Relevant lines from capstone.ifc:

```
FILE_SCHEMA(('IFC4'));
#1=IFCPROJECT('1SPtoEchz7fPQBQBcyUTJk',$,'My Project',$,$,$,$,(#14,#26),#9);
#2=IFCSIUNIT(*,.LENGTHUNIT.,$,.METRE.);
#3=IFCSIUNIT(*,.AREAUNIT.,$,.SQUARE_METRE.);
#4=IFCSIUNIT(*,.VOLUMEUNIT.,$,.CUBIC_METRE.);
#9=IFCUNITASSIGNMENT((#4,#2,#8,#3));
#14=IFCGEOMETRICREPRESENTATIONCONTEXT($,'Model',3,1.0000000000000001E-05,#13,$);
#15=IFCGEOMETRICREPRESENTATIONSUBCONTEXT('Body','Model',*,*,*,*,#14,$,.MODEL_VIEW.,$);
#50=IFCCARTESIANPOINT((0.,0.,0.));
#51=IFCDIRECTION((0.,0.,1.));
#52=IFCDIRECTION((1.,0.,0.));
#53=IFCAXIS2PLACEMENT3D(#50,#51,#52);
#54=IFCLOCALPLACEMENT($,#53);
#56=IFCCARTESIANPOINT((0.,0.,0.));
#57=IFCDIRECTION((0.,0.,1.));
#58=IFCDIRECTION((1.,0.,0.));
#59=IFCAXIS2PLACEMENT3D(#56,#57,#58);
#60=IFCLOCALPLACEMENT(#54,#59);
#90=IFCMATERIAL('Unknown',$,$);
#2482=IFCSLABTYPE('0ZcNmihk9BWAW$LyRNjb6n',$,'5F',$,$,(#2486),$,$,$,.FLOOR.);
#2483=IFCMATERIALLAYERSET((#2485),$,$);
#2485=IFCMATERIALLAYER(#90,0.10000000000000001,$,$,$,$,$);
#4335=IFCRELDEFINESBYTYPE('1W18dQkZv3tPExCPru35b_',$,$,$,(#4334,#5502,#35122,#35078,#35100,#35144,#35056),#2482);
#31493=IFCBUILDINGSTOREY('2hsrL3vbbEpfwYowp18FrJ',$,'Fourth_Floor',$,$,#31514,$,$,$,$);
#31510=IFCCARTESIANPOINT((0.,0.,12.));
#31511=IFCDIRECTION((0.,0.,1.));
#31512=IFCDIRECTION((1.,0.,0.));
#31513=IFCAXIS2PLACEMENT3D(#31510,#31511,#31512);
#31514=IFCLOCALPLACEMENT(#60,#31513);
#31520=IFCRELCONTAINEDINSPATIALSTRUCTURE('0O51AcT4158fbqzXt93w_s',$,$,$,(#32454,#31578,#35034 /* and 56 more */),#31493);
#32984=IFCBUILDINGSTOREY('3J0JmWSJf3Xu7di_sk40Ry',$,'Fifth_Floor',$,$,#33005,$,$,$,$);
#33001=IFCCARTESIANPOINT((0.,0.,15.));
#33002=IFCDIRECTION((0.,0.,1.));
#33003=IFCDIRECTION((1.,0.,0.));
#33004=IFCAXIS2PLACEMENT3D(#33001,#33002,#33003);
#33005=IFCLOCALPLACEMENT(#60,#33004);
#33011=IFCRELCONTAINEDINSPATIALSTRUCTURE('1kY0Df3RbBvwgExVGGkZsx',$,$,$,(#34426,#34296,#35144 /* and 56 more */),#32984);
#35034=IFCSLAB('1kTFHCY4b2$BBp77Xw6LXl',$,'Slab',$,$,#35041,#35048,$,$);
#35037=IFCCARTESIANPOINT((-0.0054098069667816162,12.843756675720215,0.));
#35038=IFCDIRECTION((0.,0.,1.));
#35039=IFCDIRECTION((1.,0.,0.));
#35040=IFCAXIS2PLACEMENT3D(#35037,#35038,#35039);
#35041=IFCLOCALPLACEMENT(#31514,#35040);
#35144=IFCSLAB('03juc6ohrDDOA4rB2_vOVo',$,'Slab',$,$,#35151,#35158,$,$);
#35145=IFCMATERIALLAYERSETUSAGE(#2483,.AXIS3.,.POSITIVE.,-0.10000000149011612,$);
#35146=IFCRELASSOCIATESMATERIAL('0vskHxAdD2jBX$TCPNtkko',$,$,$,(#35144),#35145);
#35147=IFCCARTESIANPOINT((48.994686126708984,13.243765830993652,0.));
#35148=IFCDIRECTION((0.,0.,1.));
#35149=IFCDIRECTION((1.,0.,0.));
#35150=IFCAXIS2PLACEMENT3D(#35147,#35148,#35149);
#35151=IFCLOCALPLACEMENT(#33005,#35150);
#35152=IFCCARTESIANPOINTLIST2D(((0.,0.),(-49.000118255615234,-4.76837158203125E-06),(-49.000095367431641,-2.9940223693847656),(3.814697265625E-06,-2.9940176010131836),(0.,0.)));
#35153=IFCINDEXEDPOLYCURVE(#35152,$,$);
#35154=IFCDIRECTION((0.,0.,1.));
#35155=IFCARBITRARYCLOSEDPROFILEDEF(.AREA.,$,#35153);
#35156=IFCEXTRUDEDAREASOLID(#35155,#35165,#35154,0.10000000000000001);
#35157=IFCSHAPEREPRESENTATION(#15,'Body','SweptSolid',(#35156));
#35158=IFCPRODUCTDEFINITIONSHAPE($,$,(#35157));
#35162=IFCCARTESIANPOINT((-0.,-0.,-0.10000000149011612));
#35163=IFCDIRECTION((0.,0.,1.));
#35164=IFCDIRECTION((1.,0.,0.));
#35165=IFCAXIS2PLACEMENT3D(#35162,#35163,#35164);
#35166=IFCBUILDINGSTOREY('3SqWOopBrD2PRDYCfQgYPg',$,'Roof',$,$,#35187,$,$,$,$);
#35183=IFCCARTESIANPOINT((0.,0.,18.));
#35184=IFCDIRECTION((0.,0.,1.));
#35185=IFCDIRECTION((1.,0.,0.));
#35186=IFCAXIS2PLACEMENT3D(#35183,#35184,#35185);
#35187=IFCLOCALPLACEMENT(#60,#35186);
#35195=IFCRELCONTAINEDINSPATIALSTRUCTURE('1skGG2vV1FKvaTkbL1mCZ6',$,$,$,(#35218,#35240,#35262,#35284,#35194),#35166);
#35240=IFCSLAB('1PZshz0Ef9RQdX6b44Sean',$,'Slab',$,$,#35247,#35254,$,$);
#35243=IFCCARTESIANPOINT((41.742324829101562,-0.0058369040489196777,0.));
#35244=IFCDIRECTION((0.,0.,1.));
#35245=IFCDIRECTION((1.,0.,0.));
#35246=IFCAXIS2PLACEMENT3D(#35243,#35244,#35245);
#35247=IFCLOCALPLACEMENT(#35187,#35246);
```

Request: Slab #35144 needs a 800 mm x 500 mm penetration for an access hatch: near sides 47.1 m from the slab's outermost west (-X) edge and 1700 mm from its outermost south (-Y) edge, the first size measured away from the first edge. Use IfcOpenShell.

```python
import numpy as np
import ifcopenshell
import ifcopenshell.api.feature
import ifcopenshell.api.geometry
import ifcopenshell.api.root
import ifcopenshell.geom
import ifcopenshell.util.placement
import ifcopenshell.util.representation
import ifcopenshell.util.shape
import ifcopenshell.util.unit

model = ifcopenshell.open("capstone.ifc")
unit_scale = ifcopenshell.util.unit.calculate_unit_scale(model)
settings = ifcopenshell.geom.settings()


def volume(element):
    """Net volume in cubic metres, openings subtracted."""
    shape = ifcopenshell.geom.create_shape(settings, element)
    return ifcopenshell.util.shape.get_volume(shape.geometry)


slab = model.by_guid("03juc6ohrDDOA4rB2_vOVo")
before = volume(slab)

# Extent in the slab's own axes, in metres. The edges named are its -X and -Y sides.
slab_shape = ifcopenshell.geom.create_shape(settings, slab)
vertices = ifcopenshell.util.shape.get_vertices(slab_shape.geometry)
x_min, y_min, bottom = vertices.min(axis=0)
top = vertices[:, 2].max()

opening = ifcopenshell.api.root.create_entity(model, ifc_class="IfcOpeningElement", name="Access hatch opening", predefined_type="OPENING")
context = ifcopenshell.util.representation.get_context(model, "Model", "Body", "MODEL_VIEW")
width, depth = 0.8, 0.5
outline = [(0.0, 0.0), (width, 0.0), (width, depth), (0.0, depth), (0.0, 0.0)]
# Overshoot both faces by 50 mm so the cut is clean.
shape = ifcopenshell.api.geometry.add_slab_representation(
    model, context=context, depth=top - bottom + 0.1, polyline=outline
)
ifcopenshell.api.geometry.assign_representation(model, product=opening, representation=shape)

matrix = ifcopenshell.util.placement.get_local_placement(slab.ObjectPlacement)
matrix[:, 3] = matrix @ np.append(np.array([x_min + 47.1, y_min + 1.7, bottom - 0.05]) / unit_scale, 1.0)
ifcopenshell.api.geometry.edit_object_placement(model, product=opening, matrix=matrix, is_si=False)
ifcopenshell.api.feature.add_feature(model, feature=opening, element=slab)

after = volume(slab)

print(f"slab volume {before:.3f} -> {after:.3f} m3")

model.write("capstone_edited.ifc")
```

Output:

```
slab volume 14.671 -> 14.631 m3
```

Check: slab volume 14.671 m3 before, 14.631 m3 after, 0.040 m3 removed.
